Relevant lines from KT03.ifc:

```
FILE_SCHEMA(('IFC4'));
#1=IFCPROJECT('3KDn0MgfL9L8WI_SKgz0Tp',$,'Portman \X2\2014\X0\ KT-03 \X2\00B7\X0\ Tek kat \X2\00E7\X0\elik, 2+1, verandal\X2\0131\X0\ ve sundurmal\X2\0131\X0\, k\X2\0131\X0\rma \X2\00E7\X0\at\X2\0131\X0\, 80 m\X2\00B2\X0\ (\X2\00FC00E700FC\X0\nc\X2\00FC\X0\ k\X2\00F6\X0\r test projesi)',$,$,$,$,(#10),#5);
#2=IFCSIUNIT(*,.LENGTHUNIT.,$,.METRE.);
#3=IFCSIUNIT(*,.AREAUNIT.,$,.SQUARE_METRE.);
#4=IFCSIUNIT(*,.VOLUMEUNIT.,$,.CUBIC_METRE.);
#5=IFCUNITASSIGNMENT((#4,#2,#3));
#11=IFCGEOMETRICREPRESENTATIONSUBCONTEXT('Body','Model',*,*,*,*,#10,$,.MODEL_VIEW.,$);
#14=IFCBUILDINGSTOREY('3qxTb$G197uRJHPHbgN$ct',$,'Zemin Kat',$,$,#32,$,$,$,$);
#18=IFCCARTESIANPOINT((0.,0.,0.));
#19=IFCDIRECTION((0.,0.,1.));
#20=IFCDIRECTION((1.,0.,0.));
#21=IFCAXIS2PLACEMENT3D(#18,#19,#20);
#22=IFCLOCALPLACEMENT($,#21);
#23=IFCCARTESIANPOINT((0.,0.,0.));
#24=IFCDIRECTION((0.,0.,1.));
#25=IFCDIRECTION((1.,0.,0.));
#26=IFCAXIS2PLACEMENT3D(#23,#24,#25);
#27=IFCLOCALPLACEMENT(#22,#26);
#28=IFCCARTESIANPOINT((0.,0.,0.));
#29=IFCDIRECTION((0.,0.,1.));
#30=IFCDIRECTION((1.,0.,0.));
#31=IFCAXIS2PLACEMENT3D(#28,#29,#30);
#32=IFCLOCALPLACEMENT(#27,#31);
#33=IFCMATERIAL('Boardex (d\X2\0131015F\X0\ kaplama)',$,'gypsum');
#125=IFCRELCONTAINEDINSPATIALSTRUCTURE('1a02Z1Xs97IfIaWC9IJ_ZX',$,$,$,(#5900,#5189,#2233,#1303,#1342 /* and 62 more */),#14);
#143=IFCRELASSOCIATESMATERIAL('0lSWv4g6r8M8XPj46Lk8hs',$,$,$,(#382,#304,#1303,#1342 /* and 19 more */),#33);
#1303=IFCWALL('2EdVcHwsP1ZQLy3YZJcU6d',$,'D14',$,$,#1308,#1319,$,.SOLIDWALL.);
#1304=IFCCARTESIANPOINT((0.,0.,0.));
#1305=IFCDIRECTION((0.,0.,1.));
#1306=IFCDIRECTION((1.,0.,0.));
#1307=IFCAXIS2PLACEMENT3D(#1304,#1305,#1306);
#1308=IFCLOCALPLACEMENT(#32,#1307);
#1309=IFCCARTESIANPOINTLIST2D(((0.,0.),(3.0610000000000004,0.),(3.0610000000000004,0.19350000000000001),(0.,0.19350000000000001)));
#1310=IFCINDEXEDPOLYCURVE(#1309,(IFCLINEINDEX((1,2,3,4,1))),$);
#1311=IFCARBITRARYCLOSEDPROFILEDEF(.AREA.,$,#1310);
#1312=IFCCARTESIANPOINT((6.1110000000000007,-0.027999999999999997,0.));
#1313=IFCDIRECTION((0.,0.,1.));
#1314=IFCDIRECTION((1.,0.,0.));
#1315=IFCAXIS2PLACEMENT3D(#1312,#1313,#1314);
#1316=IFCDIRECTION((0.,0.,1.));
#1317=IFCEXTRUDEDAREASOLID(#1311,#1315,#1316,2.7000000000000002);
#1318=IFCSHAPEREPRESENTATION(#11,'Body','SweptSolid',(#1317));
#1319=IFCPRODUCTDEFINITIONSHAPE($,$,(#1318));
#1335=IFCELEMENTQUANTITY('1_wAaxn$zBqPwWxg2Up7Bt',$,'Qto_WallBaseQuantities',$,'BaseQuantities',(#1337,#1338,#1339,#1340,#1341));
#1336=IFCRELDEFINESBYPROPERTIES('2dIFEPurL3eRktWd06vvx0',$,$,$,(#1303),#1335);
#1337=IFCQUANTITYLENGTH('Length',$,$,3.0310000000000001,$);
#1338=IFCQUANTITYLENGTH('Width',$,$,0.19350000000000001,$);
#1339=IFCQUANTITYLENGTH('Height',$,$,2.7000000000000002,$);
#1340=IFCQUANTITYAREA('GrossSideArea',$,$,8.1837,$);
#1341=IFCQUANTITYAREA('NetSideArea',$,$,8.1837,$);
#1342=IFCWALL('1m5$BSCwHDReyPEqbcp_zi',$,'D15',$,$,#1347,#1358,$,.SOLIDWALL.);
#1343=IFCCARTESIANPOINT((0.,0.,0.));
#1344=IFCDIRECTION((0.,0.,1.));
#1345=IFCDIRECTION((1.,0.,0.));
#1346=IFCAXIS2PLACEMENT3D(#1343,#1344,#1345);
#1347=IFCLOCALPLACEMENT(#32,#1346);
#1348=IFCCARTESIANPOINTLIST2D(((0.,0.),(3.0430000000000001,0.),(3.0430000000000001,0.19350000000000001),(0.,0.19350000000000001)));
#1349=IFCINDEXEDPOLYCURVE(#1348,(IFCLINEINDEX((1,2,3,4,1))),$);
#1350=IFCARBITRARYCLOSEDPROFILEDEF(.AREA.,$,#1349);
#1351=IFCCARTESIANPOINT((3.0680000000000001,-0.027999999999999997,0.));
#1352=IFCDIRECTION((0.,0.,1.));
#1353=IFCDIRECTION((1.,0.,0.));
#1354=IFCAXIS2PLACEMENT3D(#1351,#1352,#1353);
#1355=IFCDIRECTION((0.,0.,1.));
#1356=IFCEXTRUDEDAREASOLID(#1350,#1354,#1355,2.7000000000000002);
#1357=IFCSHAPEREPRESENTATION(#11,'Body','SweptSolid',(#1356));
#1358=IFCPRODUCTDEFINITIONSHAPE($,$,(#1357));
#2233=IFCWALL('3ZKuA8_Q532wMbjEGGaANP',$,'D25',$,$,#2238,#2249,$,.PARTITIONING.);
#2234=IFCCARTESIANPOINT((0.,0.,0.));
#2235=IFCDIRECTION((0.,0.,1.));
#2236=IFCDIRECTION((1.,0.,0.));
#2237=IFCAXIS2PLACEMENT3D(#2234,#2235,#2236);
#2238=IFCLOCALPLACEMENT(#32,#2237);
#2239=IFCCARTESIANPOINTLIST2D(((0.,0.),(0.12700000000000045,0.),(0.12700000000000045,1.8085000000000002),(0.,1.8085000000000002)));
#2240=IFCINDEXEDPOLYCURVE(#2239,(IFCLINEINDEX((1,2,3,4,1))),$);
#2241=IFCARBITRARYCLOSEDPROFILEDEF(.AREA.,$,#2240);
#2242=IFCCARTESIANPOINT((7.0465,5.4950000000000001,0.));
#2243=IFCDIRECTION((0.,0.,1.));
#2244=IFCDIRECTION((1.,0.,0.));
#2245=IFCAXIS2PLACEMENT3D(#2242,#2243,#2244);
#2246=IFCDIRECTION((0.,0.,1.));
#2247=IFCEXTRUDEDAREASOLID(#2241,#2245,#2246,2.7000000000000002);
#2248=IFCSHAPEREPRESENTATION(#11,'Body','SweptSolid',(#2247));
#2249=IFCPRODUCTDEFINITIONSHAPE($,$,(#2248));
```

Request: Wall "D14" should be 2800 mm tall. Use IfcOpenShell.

```python
import ifcopenshell
import ifcopenshell.api.pset
import ifcopenshell.geom
import ifcopenshell.util.element
import ifcopenshell.util.representation
import ifcopenshell.util.shape
import ifcopenshell.util.unit

model = ifcopenshell.open("KT03.ifc")
unit_scale = ifcopenshell.util.unit.calculate_unit_scale(model)
area_scale = ifcopenshell.util.unit.calculate_unit_scale(model, "AREAUNIT")
settings = ifcopenshell.geom.settings()


def volume(element):
    """Net volume in cubic metres, openings subtracted."""
    shape = ifcopenshell.geom.create_shape(settings, element)
    return ifcopenshell.util.shape.get_volume(shape.geometry)


wall = model.by_guid("2EdVcHwsP1ZQLy3YZJcU6d")
before = volume(wall)

body = ifcopenshell.util.representation.get_representation(wall, "Model", "Body")
solid = body.Items[0]
old_height = solid.Depth
solid.Depth = 2.8 / unit_scale
after = volume(wall)
thickness = 0.1935  # wall thickness in metres

# Update the stored height, areas and volumes.
qto = model.by_id(ifcopenshell.util.element.get_pset(wall, "Qto_WallBaseQuantities", should_inherit=False)["id"])
ifcopenshell.api.pset.edit_qto(model, qto=qto, properties={
    "Height": solid.Depth,
    "GrossSideArea": ifcopenshell.util.element.get_pset(wall, "Qto_WallBaseQuantities", "GrossSideArea") * solid.Depth / old_height,
    "NetSideArea": after / thickness / area_scale,
})

print(f"height {old_height:g} -> {solid.Depth:g}, volume {before:.3f} -> {after:.3f} m3")

model.write("KT03_rev.ifc")
```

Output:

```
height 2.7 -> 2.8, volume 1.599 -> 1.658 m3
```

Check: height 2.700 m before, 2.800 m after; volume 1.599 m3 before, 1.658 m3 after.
